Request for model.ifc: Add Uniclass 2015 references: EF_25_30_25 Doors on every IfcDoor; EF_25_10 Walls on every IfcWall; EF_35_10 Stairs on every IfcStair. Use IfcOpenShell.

First a look at what the model holds.

```python
import ifcopenshell

model = ifcopenshell.open("model.ifc")
print(model.schema)
print("classifications:", [c.Name for c in model.by_type("IfcClassification")])
for ifc_class in ("IfcDoor", "IfcRoof", "IfcStair", "IfcWall", "IfcWindow"):
    print(ifc_class, len(model.by_type(ifc_class)))
```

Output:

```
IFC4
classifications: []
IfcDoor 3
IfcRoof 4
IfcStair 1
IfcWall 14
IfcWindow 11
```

```python
import ifcopenshell
import ifcopenshell.api.classification

model = ifcopenshell.open("model.ifc")

system = ifcopenshell.api.classification.add_classification(model, classification="Uniclass 2015")

codes = {
    "IfcDoor": ("EF_25_30_25", "Doors"),
    "IfcWall": ("EF_25_10", "Walls"),
    "IfcStair": ("EF_35_10", "Stairs"),
}
for ifc_class, (code, name) in codes.items():
    products = model.by_type(ifc_class)
    ifcopenshell.api.classification.add_reference(
        model, products=products, classification=system, identification=code, name=name
    )
    print(code, len(products))

model.write("model_edited.ifc")
```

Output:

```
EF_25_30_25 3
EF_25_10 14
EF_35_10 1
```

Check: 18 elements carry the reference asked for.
